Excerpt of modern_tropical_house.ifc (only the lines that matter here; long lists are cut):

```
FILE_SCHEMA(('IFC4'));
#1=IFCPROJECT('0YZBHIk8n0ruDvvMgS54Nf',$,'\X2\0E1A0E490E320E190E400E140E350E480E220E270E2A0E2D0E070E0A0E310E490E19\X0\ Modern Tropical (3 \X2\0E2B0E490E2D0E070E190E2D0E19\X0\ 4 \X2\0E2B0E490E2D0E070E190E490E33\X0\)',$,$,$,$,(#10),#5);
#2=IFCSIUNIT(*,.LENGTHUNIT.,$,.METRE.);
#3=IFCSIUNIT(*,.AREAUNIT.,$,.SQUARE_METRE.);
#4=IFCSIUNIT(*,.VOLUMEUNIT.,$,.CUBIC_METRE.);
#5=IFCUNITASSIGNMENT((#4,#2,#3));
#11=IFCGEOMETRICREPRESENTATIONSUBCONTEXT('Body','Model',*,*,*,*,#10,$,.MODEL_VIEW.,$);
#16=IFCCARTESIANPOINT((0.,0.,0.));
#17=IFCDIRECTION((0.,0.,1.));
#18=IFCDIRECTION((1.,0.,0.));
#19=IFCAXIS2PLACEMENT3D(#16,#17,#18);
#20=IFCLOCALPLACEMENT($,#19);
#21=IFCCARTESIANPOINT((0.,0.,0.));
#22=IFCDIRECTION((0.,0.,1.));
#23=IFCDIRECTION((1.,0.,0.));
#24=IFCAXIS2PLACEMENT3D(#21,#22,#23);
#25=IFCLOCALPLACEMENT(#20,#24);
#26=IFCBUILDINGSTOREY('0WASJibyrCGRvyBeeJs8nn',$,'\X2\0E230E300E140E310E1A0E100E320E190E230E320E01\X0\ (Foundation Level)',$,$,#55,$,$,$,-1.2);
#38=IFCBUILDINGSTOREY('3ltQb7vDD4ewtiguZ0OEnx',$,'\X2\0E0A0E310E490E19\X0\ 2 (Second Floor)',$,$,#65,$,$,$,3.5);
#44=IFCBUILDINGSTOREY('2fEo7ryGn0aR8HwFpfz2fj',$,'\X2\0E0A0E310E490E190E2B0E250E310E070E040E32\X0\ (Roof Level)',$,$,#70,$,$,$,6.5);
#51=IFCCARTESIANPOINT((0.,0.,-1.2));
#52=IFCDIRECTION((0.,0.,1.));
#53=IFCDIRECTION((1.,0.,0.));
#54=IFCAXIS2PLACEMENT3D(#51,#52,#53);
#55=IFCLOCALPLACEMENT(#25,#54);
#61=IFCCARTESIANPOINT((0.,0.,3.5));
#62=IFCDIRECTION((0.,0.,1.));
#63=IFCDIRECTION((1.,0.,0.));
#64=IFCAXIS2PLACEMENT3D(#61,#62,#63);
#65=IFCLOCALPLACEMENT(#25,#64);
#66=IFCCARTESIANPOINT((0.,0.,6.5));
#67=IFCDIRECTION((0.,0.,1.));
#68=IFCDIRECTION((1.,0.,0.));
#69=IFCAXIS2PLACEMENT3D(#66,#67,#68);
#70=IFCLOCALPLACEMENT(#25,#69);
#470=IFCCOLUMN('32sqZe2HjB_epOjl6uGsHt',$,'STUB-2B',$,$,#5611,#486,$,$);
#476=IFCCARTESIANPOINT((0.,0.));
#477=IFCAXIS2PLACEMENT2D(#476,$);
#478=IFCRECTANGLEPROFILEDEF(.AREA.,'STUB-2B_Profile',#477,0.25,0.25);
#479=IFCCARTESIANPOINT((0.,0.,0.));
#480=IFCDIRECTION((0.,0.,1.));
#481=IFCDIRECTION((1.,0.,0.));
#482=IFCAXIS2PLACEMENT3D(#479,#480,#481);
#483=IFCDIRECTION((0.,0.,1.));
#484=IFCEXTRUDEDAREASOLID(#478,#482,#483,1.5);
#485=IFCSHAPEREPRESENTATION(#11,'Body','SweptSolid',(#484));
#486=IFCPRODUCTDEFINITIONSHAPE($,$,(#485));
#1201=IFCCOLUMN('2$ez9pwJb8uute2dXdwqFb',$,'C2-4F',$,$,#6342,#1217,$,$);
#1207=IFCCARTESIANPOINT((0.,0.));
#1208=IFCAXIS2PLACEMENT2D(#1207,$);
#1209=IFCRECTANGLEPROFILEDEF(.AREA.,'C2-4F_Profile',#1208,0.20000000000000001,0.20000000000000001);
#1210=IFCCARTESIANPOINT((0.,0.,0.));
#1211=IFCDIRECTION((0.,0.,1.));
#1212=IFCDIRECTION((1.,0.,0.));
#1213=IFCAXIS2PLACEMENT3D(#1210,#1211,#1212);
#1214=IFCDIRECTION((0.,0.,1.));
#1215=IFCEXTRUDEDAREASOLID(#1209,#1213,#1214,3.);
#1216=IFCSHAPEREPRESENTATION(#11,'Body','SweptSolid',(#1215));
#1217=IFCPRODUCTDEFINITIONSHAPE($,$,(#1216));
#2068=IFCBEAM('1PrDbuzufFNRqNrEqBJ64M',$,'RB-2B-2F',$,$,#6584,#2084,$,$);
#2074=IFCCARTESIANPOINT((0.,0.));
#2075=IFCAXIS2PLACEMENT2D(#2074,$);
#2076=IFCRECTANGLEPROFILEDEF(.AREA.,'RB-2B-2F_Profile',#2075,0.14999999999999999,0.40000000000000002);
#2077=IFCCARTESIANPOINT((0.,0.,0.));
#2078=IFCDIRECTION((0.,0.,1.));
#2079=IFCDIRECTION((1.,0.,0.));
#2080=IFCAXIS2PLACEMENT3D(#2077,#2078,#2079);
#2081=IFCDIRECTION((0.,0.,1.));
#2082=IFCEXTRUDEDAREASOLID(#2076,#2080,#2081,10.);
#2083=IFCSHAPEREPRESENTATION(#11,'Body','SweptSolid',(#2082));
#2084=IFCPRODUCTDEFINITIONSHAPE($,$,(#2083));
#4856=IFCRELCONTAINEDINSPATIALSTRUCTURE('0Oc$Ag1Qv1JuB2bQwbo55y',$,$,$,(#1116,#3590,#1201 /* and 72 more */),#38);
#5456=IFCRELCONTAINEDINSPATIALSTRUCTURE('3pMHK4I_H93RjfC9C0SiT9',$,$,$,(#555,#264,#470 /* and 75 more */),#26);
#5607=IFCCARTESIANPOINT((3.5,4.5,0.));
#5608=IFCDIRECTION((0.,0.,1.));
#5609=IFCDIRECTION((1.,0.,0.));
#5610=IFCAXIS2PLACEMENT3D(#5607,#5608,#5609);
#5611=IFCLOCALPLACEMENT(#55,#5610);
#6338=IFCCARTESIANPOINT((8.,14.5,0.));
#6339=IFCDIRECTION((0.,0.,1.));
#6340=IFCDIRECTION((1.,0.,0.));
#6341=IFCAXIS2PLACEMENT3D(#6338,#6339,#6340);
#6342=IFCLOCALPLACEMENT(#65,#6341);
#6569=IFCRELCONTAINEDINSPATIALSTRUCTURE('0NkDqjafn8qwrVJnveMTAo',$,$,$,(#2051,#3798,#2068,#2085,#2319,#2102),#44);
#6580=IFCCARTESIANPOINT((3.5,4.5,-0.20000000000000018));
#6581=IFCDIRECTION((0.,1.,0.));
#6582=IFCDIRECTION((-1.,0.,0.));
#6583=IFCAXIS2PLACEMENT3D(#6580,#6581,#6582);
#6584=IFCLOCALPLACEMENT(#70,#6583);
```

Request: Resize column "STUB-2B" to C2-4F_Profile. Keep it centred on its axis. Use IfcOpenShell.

```python
import ifcopenshell
import ifcopenshell.util.element
import ifcopenshell.util.representation

model = ifcopenshell.open("modern_tropical_house.ifc")

member = model.by_id(470)
source = next(p for p in model.by_type("IfcRectangleProfileDef") if p.ProfileName == "C2-4F_Profile")

body = ifcopenshell.util.representation.get_representation(member, "Model", "Body")
solid = body.Items[0]
old_profile = solid.SweptArea

# Copy the section's sizes but keep this member's own profile position.
profile = ifcopenshell.util.element.copy(model, source)
profile.Position = old_profile.Position
solid.SweptArea = profile
if not model.get_total_inverses(old_profile):
    ifcopenshell.util.element.remove_deep2(model, old_profile)

print(solid.SweptArea)

model.write("modern_tropical_house_rev.ifc")
```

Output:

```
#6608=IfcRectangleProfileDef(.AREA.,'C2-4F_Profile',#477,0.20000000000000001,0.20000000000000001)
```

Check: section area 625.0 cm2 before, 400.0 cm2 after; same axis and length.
